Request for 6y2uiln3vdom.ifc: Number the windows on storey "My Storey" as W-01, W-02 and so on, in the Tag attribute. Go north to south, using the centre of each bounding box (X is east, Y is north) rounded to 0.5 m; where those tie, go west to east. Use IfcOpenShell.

First a look at what the model holds.

```python
import ifcopenshell
import ifcopenshell.util.element
import ifcopenshell.util.placement

model = ifcopenshell.open("6y2uiln3vdom.ifc")
print(model.schema)
storey = next(s for s in model.by_type("IfcBuildingStorey") if s.Name == "My Storey")
windows = [e for e in ifcopenshell.util.element.get_decomposition(storey) if e.is_a("IfcWindow")]
for e in sorted(windows, key=lambda e: e.id()):
    origin = ifcopenshell.util.placement.get_local_placement(e.ObjectPlacement)[:3, 3]
    print(e.id(), e.Tag, e.Name, origin.round(2) + 0.0, sep=" | ")
```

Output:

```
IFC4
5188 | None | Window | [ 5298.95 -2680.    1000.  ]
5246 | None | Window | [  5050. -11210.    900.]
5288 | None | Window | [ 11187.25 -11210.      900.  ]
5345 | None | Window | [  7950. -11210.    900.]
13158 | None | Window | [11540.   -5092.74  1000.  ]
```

```python
import ifcopenshell
import ifcopenshell.geom
import ifcopenshell.util.element
import ifcopenshell.util.shape

model = ifcopenshell.open("6y2uiln3vdom.ifc")
settings = ifcopenshell.geom.settings()
settings.set("use-world-coords", True)


def centre(element):
    shape = ifcopenshell.geom.create_shape(settings, element)
    return ifcopenshell.util.shape.get_bbox_centroid(shape.geometry)


storey = next(s for s in model.by_type("IfcBuildingStorey") if s.Name == "My Storey")
windows = [e for e in ifcopenshell.util.element.get_decomposition(storey) if e.is_a("IfcWindow")]

# Insertion points can sit at a corner or the storey origin, so sort by the geometry (in metres).
centres = {e: centre(e) for e in windows}
windows.sort(key=lambda e: (-round(centres[e][1] / 0.5), centres[e][0]))

for i, e in enumerate(windows, start=1):
    number = f"W-{i:02d}"
    e.Tag = number
    print(e.id(), number)

model.write("6y2uiln3vdom-out.ifc")
```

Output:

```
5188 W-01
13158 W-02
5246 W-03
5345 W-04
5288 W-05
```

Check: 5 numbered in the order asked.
